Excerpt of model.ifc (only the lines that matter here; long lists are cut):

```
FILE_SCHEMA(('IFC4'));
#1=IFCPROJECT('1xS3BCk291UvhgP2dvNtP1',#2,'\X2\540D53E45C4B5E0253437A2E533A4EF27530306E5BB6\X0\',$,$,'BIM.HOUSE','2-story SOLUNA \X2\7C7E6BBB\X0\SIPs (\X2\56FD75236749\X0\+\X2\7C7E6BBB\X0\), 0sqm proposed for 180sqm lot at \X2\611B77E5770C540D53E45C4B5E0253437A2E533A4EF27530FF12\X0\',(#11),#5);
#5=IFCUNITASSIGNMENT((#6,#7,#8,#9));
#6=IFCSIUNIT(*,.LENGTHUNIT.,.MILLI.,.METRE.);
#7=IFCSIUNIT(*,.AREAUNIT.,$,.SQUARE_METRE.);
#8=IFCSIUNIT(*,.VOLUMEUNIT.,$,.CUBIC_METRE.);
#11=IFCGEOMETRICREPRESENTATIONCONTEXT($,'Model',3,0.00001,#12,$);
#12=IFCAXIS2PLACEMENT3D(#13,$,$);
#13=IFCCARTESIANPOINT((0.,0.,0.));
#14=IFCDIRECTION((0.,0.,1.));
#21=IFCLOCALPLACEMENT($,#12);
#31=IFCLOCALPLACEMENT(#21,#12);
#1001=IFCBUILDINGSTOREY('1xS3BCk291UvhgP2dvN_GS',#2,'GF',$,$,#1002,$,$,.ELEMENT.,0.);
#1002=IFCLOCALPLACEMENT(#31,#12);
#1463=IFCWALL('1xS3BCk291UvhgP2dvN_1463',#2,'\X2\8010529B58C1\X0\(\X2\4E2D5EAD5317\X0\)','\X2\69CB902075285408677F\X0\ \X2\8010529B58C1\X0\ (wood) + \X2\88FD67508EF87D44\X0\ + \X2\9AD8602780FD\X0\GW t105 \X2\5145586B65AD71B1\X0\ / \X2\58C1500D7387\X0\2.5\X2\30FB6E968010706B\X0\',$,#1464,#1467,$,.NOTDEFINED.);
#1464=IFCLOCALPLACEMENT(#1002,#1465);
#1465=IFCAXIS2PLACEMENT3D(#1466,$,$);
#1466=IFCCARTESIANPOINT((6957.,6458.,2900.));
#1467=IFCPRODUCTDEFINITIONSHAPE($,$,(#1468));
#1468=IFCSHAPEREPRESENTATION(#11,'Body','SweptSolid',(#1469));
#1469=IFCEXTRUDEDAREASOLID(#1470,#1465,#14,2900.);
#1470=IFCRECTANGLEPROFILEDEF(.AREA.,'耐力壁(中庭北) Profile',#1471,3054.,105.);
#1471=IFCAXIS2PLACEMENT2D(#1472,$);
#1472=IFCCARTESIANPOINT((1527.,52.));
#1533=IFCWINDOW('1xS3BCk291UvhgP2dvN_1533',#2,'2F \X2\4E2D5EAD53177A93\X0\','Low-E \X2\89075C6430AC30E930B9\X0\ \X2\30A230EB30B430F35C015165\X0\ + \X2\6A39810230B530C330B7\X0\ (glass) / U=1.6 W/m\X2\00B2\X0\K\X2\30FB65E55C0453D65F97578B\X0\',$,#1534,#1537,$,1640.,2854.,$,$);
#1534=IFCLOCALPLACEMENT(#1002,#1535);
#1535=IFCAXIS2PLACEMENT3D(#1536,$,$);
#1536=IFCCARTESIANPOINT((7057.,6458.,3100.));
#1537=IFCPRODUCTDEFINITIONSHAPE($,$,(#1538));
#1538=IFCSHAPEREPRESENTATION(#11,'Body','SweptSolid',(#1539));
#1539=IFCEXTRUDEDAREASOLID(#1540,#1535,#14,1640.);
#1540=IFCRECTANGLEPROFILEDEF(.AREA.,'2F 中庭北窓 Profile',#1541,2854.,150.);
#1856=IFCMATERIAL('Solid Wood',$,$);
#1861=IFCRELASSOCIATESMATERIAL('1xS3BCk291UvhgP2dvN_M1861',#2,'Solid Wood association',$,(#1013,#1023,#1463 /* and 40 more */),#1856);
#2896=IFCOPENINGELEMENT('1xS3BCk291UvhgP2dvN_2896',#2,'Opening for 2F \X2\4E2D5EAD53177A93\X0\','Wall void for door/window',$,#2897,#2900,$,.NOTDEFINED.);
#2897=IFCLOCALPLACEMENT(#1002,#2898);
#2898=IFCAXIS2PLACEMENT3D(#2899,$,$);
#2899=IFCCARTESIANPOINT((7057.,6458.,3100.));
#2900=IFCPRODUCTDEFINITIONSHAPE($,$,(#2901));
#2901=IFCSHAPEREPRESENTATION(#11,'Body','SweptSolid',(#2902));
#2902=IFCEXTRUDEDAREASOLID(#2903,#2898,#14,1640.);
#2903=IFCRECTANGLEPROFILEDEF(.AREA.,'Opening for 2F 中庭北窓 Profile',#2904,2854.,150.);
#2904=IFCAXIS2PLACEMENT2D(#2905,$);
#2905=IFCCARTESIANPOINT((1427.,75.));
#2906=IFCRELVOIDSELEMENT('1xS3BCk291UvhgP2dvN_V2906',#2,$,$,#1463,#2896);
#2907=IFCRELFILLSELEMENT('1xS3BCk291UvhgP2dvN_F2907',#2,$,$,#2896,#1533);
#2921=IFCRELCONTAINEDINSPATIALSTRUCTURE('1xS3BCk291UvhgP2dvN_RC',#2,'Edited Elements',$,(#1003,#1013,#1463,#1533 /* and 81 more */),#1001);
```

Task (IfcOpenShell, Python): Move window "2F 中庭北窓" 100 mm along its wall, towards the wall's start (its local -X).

```python
import ifcopenshell
import ifcopenshell.api.geometry
import ifcopenshell.util.placement

model = ifcopenshell.open("model.ifc")

window = model.by_guid("1xS3BCk291UvhgP2dvN_1533")
opening = window.FillsVoids[0].RelatingOpeningElement
wall = opening.VoidsElements[0].RelatingBuildingElement

wall_matrix = ifcopenshell.util.placement.get_local_placement(wall.ObjectPlacement)
shift = wall_matrix[:3, 0] * -100.0
before = ifcopenshell.util.placement.get_local_placement(window.ObjectPlacement)[:3, 3].copy()

# The window is not placed relative to its opening, so move both.
for product in (opening, window):
    matrix = ifcopenshell.util.placement.get_local_placement(product.ObjectPlacement)
    matrix[:3, 3] += shift
    ifcopenshell.api.geometry.edit_object_placement(model, product=product, matrix=matrix, is_si=False)

after = ifcopenshell.util.placement.get_local_placement(window.ObjectPlacement)[:3, 3]
print("window moved by", (after - before).round(3) + 0.0)

model.write("model-out.ifc")
```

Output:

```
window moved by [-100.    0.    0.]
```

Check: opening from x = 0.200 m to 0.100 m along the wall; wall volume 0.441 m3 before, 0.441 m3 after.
